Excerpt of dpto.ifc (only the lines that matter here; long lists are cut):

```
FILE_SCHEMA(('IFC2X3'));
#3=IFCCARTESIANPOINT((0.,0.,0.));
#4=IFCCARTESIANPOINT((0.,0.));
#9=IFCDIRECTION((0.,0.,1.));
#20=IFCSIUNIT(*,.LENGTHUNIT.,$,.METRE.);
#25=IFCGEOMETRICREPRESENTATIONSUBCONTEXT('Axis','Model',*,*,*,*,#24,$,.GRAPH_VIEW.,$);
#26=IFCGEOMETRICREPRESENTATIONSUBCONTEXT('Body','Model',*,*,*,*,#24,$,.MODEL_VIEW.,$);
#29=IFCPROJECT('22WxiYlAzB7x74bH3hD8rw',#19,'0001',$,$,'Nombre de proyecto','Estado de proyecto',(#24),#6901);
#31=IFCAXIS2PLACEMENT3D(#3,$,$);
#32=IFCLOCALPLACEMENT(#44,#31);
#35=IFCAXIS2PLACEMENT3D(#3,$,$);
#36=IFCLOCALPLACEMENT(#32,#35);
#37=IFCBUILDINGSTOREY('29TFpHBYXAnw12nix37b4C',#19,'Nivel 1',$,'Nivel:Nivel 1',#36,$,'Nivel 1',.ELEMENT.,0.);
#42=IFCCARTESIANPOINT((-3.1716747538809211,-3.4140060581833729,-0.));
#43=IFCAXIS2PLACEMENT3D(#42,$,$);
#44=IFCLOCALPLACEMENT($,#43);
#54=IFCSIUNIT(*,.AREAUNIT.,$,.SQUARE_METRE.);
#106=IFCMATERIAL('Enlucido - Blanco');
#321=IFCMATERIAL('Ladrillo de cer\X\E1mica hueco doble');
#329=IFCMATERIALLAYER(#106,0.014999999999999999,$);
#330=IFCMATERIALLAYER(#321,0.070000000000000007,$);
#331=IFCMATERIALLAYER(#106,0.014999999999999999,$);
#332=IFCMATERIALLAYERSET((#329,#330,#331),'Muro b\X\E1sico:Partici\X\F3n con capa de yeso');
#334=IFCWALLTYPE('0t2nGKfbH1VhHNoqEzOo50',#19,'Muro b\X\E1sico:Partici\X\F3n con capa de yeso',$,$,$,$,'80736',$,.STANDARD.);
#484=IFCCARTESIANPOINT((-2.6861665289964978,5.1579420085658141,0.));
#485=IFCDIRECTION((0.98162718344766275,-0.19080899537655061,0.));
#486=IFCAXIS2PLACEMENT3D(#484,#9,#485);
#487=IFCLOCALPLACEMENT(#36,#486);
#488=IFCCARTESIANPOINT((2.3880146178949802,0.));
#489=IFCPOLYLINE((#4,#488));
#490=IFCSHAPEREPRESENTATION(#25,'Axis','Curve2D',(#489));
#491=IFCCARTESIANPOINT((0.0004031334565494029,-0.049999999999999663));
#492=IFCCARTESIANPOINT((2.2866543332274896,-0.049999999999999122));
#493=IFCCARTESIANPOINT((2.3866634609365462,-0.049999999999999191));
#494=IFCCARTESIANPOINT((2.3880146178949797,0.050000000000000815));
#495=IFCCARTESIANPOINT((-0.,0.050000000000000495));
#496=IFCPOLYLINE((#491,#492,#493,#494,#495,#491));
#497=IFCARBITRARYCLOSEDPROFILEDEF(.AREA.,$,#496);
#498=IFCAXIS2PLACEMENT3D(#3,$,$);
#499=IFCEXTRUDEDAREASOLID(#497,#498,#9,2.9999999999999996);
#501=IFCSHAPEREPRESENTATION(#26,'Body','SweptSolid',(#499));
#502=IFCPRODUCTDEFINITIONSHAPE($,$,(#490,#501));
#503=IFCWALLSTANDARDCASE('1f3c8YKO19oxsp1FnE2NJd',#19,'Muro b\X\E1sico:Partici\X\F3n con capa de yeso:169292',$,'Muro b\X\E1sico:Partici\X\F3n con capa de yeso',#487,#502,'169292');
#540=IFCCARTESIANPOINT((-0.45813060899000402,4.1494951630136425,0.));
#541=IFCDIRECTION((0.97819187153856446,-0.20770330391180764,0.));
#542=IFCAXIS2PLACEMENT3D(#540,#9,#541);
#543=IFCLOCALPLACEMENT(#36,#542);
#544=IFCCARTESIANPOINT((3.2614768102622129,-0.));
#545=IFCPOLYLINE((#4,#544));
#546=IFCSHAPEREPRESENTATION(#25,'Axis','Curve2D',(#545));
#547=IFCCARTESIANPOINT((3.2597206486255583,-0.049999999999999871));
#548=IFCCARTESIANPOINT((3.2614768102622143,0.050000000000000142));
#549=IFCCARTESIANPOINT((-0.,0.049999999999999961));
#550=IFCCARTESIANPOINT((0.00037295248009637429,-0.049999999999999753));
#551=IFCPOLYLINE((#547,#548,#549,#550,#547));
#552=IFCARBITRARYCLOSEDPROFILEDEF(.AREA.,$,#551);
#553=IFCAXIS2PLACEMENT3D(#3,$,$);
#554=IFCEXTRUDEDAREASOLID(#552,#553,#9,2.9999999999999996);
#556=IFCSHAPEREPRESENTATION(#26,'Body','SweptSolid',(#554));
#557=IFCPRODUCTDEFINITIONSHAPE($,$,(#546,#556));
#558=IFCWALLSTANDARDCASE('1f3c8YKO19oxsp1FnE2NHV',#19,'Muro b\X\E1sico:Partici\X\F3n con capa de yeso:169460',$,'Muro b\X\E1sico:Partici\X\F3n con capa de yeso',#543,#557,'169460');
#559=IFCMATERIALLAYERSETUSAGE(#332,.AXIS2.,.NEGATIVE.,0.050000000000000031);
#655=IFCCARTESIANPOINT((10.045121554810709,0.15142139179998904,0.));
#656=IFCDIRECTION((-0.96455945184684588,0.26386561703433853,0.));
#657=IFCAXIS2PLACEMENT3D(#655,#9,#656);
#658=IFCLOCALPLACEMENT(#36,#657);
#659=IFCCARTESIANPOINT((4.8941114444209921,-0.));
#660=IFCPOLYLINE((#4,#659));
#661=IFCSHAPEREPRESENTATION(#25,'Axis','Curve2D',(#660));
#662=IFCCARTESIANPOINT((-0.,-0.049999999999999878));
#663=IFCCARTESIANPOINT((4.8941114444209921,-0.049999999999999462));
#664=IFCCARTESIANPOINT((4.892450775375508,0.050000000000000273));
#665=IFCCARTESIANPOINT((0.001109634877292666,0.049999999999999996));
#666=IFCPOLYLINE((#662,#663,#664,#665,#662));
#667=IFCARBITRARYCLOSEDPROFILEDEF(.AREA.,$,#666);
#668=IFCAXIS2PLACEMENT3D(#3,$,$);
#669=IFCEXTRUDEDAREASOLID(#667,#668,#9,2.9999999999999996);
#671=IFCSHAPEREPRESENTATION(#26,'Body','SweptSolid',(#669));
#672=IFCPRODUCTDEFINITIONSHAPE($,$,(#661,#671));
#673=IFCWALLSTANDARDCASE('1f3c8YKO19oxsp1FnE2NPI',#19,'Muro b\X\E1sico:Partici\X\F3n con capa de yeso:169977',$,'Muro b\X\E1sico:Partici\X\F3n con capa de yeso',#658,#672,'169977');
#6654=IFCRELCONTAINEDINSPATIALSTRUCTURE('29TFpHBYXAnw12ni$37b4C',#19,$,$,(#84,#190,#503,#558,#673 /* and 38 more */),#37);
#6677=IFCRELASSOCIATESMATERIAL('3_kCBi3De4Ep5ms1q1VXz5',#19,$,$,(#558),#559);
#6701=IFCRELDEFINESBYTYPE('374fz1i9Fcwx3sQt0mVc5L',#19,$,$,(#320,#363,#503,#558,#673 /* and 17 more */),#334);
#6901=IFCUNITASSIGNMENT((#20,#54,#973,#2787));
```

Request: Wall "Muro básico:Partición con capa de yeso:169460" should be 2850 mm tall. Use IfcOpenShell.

```python
import ifcopenshell
import ifcopenshell.geom
import ifcopenshell.util.representation
import ifcopenshell.util.shape
import ifcopenshell.util.unit

model = ifcopenshell.open("dpto.ifc")
unit_scale = ifcopenshell.util.unit.calculate_unit_scale(model)
settings = ifcopenshell.geom.settings()


def volume(element):
    """Net volume in cubic metres, openings subtracted."""
    shape = ifcopenshell.geom.create_shape(settings, element)
    return ifcopenshell.util.shape.get_volume(shape.geometry)


wall = model.by_guid("1f3c8YKO19oxsp1FnE2NHV")
before = volume(wall)

body = ifcopenshell.util.representation.get_representation(wall, "Model", "Body")
solid = body.Items[0]
old_height = solid.Depth
solid.Depth = 2.85 / unit_scale
after = volume(wall)

print(f"height {old_height:g} -> {solid.Depth:g}, volume {before:.3f} -> {after:.3f} m3")

model.write("dpto_v2.ifc")
```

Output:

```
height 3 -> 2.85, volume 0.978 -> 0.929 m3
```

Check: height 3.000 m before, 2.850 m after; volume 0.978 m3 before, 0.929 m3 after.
